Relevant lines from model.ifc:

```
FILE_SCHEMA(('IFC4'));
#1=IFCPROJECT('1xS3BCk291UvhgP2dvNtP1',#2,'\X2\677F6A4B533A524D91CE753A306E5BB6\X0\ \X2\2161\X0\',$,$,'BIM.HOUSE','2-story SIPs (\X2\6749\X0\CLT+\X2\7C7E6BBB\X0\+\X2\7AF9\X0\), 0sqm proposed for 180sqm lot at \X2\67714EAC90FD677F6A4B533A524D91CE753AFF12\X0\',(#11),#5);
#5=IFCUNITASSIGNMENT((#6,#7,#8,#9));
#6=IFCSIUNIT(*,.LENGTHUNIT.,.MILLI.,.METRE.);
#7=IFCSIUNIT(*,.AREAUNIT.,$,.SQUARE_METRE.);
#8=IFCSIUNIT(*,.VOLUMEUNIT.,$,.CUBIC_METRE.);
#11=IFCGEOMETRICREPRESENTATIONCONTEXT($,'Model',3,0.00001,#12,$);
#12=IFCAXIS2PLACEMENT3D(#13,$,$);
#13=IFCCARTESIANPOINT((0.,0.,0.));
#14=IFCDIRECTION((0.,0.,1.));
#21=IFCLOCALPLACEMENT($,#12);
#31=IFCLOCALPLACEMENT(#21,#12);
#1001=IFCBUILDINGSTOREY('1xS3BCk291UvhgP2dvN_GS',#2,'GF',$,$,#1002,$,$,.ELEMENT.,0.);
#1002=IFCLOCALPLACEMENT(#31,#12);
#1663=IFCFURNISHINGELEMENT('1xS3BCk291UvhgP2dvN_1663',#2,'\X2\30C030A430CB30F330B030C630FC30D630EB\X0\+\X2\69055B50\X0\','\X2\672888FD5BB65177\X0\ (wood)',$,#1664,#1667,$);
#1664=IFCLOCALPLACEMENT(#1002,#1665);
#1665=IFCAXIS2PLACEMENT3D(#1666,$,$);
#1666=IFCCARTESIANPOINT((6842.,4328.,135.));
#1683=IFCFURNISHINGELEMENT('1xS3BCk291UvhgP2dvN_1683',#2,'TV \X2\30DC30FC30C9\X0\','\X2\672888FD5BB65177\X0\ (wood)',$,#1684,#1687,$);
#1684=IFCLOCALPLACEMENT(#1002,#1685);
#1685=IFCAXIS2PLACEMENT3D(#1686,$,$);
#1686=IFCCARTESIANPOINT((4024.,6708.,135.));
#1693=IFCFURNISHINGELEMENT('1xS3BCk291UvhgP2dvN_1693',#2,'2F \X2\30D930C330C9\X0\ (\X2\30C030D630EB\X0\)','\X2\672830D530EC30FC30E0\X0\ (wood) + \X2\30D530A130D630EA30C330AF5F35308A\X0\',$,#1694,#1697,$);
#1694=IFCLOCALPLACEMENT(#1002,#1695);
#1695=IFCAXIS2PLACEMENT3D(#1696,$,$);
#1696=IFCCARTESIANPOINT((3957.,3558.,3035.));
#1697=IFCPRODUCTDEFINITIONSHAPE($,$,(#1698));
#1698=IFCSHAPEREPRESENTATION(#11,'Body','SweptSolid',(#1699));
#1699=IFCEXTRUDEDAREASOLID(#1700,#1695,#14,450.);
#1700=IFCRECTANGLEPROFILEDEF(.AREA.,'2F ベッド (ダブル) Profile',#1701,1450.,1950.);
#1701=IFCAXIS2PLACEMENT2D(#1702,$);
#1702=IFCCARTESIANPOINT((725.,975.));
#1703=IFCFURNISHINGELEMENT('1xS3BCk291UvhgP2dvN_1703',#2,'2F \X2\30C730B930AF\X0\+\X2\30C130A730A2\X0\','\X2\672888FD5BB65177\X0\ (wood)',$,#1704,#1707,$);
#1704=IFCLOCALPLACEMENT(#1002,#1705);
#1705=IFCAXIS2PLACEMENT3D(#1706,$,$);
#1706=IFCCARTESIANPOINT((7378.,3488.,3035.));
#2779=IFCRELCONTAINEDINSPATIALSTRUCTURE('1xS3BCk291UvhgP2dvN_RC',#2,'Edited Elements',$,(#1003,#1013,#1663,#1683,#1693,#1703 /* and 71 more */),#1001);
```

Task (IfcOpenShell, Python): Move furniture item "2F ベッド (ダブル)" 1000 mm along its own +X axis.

```python
import ifcopenshell
import ifcopenshell.api.geometry
import ifcopenshell.util.placement

model = ifcopenshell.open("model.ifc")

item = model.by_id(1693)
matrix = ifcopenshell.util.placement.get_local_placement(item.ObjectPlacement)
matrix[:3, 3] += matrix[:3, 0] * 1000.0
ifcopenshell.api.geometry.edit_object_placement(model, product=item, matrix=matrix, is_si=False)

print(ifcopenshell.util.placement.get_local_placement(item.ObjectPlacement).round(3) + 0.0)

model.write("model_updated.ifc")
```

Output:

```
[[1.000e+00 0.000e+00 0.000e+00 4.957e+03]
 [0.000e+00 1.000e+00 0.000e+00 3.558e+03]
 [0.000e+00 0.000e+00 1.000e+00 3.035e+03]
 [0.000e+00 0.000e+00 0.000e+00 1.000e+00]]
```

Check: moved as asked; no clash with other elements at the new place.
